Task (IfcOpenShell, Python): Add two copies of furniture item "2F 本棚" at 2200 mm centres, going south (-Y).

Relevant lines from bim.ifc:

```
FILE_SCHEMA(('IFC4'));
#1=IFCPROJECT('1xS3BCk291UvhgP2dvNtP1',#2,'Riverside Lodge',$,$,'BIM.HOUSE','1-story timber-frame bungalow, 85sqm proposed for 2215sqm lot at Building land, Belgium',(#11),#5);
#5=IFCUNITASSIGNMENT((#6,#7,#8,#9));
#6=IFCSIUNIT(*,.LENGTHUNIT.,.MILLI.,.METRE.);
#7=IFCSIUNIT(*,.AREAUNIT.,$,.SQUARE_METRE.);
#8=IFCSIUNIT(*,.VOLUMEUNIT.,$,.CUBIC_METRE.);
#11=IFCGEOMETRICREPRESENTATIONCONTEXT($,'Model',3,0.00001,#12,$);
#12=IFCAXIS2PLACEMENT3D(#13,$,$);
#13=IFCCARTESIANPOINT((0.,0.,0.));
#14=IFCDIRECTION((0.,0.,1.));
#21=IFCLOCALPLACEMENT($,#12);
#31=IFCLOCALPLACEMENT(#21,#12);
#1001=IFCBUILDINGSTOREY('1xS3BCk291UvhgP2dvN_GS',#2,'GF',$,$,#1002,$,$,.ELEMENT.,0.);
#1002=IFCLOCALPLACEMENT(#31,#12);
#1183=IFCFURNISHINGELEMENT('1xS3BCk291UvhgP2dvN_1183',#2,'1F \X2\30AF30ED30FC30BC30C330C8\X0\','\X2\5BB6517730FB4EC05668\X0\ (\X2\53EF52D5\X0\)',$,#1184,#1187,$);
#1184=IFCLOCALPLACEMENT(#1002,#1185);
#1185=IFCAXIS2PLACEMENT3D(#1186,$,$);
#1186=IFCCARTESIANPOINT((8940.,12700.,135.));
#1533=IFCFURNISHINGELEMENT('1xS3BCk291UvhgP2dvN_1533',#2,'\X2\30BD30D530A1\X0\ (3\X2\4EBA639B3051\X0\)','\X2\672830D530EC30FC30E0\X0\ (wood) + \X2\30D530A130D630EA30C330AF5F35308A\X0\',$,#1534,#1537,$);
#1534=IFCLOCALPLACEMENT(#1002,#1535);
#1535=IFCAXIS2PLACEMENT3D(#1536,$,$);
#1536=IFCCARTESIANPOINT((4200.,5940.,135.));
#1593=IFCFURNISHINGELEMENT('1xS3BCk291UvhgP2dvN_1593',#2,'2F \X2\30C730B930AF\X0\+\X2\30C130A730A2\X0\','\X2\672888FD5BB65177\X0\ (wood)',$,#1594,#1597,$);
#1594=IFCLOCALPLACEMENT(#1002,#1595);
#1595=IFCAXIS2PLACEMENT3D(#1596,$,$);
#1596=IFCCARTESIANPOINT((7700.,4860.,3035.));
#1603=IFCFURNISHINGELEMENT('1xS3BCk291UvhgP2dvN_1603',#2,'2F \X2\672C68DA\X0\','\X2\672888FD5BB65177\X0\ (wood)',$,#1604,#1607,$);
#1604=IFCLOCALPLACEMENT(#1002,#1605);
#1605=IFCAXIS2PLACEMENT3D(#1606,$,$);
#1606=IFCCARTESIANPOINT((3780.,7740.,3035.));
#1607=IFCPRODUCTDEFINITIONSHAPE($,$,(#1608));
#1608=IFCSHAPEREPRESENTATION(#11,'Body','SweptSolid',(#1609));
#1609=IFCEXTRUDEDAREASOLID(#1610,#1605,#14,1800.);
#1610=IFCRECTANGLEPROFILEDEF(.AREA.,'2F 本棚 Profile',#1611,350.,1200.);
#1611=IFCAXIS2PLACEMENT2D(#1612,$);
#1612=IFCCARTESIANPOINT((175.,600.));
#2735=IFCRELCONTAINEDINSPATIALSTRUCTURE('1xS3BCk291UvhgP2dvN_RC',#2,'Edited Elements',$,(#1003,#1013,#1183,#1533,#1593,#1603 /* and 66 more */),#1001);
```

```python
import numpy as np
import ifcopenshell
import ifcopenshell.api.geometry
import ifcopenshell.api.root
import ifcopenshell.util.element
import ifcopenshell.util.placement

model = ifcopenshell.open("bim.ifc")


def reuse_history(source, copy):
    """copy_class also copies each property set's owner history, people and application; keep the originals."""
    for rel in copy.IsDefinedBy:
        if rel.is_a("IfcRelDefinesByProperties") and (history := rel.RelatingPropertyDefinition.OwnerHistory):
            rel.RelatingPropertyDefinition.OwnerHistory = source.OwnerHistory
            ifcopenshell.util.element.remove_deep2(model, history)


source = model.by_guid("1xS3BCk291UvhgP2dvN_1603")
base = ifcopenshell.util.placement.get_local_placement(source.ObjectPlacement)
step = np.array([0.0, -1.0, 0.0]) * 2200.0

for i in range(1, 3):
    copy = ifcopenshell.api.root.copy_class(model, product=source)
    copy.Representation = ifcopenshell.util.element.copy_deep(
        model, source.Representation, exclude=["IfcGeometricRepresentationContext", "IfcRepresentationMap"]
    )
    reuse_history(source, copy)
    matrix = base.copy()
    matrix[:3, 3] += i * step
    print("added at", matrix[:3, 3].round(3) + 0.0)
    ifcopenshell.api.geometry.edit_object_placement(model, product=copy, matrix=matrix, is_si=False)

model.write("bim_updated.ifc")
```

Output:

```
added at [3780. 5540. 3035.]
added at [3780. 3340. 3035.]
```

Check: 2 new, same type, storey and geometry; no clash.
